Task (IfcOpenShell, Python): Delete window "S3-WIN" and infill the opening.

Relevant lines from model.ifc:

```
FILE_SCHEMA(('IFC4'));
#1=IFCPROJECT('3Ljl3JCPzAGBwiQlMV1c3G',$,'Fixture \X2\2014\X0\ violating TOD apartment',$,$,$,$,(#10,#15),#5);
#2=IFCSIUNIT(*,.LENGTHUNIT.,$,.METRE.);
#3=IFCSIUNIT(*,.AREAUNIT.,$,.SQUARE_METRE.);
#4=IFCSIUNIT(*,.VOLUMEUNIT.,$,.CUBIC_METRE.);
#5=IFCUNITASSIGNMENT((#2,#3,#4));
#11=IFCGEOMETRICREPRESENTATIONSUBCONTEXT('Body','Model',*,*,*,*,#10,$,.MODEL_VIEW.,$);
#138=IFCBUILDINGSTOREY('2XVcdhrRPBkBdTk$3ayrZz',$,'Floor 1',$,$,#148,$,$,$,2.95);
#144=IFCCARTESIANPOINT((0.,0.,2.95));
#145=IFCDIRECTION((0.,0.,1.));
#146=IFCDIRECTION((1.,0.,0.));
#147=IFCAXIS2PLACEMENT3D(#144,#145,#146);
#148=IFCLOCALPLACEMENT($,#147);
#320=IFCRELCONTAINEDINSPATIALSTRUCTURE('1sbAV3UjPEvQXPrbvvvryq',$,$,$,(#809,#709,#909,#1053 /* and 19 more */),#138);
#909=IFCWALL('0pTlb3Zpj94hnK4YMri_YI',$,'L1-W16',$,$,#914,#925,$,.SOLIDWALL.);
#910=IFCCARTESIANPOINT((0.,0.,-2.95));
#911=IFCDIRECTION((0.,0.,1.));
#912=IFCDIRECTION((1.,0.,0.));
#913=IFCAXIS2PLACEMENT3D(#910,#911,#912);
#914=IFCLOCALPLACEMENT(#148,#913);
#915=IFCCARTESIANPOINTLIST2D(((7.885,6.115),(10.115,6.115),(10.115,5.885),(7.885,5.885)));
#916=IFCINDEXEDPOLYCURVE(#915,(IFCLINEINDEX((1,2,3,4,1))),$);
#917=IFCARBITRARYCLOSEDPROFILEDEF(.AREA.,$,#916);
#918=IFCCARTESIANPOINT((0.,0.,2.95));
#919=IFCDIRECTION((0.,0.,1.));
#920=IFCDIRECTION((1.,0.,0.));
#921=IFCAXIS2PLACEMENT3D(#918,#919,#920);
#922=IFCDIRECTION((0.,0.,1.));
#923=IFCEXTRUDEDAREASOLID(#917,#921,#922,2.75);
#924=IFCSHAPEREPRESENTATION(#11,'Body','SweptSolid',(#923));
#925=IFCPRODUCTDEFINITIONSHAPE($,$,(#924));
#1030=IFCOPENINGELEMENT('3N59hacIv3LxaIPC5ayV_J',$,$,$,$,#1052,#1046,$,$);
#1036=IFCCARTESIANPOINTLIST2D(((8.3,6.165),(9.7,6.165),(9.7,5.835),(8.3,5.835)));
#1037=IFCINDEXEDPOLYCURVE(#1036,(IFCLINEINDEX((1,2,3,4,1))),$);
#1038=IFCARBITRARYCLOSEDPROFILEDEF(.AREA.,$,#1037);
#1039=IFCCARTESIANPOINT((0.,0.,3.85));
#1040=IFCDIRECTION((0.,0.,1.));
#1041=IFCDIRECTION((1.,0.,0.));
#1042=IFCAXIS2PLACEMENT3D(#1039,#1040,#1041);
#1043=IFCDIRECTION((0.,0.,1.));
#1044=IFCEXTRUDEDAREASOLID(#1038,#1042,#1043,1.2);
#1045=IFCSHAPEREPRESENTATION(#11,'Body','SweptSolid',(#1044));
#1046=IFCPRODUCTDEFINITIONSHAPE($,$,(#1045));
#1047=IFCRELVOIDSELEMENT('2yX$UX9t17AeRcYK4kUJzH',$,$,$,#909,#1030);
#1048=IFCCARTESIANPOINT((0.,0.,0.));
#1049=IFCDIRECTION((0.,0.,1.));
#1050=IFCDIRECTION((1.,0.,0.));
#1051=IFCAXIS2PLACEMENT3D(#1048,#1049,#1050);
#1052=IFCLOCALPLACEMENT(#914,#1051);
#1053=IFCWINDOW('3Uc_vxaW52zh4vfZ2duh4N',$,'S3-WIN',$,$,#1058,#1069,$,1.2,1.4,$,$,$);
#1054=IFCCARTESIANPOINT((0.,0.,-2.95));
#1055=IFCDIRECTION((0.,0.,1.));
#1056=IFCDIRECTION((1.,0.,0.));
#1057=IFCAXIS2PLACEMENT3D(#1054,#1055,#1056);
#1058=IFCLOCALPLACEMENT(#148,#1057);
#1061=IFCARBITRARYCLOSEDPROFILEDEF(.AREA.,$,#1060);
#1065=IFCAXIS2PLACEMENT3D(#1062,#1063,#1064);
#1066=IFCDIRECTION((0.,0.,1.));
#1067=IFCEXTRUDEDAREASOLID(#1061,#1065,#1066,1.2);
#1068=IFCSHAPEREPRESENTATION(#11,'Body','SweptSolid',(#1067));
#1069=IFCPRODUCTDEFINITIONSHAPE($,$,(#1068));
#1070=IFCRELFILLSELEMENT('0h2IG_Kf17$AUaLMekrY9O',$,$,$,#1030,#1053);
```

```python
import ifcopenshell
import ifcopenshell.api.feature
import ifcopenshell.api.root
import ifcopenshell.geom
import ifcopenshell.util.shape

model = ifcopenshell.open("model.ifc")
settings = ifcopenshell.geom.settings()


def volume(element):
    """Net volume in cubic metres, openings subtracted."""
    shape = ifcopenshell.geom.create_shape(settings, element)
    return ifcopenshell.util.shape.get_volume(shape.geometry)


window = model.by_id(1053)
opening = window.FillsVoids[0].RelatingOpeningElement
wall = opening.VoidsElements[0].RelatingBuildingElement
before = volume(wall)

ifcopenshell.api.root.remove_product(model, product=window)
ifcopenshell.api.feature.remove_feature(model, feature=opening)

after = volume(wall)

print(f"wall volume {before:.3f} -> {after:.3f} m3")

model.write("model_edited.ifc")
```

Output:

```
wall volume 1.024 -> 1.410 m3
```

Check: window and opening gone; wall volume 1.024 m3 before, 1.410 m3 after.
